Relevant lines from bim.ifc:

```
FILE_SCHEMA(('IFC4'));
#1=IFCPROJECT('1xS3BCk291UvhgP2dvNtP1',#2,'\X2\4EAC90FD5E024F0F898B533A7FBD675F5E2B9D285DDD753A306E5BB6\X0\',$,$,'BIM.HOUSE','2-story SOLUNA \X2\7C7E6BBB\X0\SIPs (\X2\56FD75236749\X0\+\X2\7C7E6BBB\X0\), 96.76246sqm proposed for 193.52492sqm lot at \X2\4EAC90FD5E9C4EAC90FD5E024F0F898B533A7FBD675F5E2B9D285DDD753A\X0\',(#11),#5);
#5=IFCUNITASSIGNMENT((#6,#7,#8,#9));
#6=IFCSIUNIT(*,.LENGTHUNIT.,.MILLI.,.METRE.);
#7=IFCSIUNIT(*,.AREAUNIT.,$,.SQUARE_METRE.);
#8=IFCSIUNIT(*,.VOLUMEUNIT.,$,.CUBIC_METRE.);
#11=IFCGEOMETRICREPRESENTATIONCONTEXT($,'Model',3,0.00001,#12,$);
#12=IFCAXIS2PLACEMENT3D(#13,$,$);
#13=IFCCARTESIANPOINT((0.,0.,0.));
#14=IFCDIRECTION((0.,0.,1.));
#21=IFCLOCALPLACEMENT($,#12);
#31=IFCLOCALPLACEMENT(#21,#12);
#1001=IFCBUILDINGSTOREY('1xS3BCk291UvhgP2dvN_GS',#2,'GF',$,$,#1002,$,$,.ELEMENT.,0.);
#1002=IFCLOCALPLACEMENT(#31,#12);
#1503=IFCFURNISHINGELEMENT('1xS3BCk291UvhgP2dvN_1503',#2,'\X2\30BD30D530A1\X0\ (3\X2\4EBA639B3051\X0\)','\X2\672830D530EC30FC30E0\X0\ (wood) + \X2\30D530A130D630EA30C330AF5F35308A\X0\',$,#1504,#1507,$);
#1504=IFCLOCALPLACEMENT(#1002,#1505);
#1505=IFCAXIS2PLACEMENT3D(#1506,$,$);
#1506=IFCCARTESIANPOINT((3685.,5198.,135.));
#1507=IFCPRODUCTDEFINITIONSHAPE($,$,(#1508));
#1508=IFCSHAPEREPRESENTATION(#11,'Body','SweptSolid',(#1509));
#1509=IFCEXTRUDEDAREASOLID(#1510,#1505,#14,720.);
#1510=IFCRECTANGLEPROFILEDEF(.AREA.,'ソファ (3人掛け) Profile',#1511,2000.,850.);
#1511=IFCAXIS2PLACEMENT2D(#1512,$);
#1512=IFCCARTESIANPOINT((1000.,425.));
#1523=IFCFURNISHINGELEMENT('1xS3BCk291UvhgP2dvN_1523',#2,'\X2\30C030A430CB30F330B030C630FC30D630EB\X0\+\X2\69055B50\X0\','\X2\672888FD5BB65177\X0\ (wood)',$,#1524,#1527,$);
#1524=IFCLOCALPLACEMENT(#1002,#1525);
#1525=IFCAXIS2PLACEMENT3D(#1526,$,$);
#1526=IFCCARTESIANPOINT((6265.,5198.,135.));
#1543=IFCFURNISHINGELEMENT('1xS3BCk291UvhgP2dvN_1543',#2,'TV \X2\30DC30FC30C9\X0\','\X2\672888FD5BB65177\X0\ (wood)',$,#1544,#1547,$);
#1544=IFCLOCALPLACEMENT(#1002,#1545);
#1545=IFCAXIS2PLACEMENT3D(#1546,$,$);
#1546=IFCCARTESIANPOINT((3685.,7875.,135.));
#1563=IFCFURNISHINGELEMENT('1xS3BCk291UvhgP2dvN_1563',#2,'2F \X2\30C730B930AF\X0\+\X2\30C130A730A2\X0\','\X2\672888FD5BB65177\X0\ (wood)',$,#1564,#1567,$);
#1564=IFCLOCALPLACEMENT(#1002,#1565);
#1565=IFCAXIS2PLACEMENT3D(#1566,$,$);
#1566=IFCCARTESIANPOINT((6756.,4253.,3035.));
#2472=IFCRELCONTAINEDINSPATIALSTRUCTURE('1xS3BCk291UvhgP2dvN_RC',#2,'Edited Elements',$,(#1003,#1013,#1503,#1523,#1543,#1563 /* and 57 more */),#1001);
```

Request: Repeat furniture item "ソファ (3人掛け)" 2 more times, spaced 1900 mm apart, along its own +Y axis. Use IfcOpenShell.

```python
import ifcopenshell
import ifcopenshell.api.geometry
import ifcopenshell.api.root
import ifcopenshell.util.element
import ifcopenshell.util.placement

model = ifcopenshell.open("bim.ifc")


def reuse_history(source, copy):
    """copy_class also copies each property set's owner history, people and application; keep the originals."""
    for rel in copy.IsDefinedBy:
        if rel.is_a("IfcRelDefinesByProperties") and (history := rel.RelatingPropertyDefinition.OwnerHistory):
            rel.RelatingPropertyDefinition.OwnerHistory = source.OwnerHistory
            ifcopenshell.util.element.remove_deep2(model, history)


source = model.by_id(1503)
base = ifcopenshell.util.placement.get_local_placement(source.ObjectPlacement)
step = base[:3, 1] * 1900.0

for i in range(1, 3):
    copy = ifcopenshell.api.root.copy_class(model, product=source)
    copy.Representation = ifcopenshell.util.element.copy_deep(
        model, source.Representation, exclude=["IfcGeometricRepresentationContext", "IfcRepresentationMap"]
    )
    reuse_history(source, copy)
    matrix = base.copy()
    matrix[:3, 3] += i * step
    print("added at", matrix[:3, 3].round(3) + 0.0)
    ifcopenshell.api.geometry.edit_object_placement(model, product=copy, matrix=matrix, is_si=False)

model.write("bim_edited.ifc")
```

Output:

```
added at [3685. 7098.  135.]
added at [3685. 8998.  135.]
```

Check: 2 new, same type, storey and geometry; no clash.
